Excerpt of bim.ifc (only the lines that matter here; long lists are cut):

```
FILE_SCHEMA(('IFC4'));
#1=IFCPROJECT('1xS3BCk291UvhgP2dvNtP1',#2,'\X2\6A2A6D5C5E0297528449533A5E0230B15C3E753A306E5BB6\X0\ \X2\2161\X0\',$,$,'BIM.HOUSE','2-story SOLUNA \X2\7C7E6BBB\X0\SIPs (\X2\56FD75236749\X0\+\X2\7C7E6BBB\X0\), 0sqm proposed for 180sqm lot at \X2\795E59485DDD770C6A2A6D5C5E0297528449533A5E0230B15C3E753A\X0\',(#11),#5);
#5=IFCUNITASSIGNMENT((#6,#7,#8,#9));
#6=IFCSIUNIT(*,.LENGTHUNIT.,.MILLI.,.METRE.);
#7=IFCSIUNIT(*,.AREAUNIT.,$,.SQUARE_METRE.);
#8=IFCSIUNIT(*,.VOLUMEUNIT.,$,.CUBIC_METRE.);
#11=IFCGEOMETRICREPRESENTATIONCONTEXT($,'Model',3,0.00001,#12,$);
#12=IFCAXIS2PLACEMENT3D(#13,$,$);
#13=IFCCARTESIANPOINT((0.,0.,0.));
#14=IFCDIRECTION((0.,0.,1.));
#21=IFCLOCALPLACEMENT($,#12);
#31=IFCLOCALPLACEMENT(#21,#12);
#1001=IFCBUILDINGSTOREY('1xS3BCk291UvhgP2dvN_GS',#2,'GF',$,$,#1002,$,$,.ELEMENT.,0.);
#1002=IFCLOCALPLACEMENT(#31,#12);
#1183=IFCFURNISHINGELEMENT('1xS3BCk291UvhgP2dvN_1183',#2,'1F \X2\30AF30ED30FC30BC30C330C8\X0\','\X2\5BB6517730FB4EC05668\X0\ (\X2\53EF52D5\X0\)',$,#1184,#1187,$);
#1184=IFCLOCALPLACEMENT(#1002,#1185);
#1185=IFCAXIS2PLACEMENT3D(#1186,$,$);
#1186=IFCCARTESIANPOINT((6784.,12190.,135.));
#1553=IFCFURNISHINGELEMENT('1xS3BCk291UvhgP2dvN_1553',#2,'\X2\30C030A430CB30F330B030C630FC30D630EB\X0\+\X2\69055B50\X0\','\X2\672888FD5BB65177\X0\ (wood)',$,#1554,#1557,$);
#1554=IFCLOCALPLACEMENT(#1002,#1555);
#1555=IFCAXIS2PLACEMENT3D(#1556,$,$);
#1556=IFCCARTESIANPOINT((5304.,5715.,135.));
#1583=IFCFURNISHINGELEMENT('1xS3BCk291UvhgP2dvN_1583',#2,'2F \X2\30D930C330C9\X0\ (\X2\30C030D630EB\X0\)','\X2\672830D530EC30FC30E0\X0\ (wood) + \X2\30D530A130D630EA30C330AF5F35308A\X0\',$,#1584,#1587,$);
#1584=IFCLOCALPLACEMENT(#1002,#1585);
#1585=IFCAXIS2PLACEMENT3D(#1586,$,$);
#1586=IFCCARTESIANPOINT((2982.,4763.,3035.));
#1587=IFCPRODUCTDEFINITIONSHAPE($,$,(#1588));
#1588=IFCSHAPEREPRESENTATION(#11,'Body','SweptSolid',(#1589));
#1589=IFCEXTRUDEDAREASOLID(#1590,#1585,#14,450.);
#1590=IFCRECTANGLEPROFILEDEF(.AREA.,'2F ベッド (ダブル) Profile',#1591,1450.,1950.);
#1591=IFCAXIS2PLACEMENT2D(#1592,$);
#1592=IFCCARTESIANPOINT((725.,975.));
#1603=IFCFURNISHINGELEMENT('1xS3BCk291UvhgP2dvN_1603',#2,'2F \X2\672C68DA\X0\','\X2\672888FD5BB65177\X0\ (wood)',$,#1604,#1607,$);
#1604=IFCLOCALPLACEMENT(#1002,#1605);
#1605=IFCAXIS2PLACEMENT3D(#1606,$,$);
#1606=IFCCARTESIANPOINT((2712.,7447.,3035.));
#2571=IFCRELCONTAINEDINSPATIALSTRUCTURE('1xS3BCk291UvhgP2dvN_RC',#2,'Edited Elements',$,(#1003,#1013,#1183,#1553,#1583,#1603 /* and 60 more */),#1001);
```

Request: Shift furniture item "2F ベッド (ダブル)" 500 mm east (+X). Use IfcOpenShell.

```python
import ifcopenshell
import ifcopenshell.api.geometry
import ifcopenshell.util.placement
import ifcopenshell.util.unit

model = ifcopenshell.open("bim.ifc")
unit_scale = ifcopenshell.util.unit.calculate_unit_scale(model)

item = model.by_id(1583)
matrix = ifcopenshell.util.placement.get_local_placement(item.ObjectPlacement)
matrix[0, 3] += 0.5 / unit_scale
ifcopenshell.api.geometry.edit_object_placement(model, product=item, matrix=matrix, is_si=False)

print(ifcopenshell.util.placement.get_local_placement(item.ObjectPlacement).round(3) + 0.0)

model.write("bim-out.ifc")
```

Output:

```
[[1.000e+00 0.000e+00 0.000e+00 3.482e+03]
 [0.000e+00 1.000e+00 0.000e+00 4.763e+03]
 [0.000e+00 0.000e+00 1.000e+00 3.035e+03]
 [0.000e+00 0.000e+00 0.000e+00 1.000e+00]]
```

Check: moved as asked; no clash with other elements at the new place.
